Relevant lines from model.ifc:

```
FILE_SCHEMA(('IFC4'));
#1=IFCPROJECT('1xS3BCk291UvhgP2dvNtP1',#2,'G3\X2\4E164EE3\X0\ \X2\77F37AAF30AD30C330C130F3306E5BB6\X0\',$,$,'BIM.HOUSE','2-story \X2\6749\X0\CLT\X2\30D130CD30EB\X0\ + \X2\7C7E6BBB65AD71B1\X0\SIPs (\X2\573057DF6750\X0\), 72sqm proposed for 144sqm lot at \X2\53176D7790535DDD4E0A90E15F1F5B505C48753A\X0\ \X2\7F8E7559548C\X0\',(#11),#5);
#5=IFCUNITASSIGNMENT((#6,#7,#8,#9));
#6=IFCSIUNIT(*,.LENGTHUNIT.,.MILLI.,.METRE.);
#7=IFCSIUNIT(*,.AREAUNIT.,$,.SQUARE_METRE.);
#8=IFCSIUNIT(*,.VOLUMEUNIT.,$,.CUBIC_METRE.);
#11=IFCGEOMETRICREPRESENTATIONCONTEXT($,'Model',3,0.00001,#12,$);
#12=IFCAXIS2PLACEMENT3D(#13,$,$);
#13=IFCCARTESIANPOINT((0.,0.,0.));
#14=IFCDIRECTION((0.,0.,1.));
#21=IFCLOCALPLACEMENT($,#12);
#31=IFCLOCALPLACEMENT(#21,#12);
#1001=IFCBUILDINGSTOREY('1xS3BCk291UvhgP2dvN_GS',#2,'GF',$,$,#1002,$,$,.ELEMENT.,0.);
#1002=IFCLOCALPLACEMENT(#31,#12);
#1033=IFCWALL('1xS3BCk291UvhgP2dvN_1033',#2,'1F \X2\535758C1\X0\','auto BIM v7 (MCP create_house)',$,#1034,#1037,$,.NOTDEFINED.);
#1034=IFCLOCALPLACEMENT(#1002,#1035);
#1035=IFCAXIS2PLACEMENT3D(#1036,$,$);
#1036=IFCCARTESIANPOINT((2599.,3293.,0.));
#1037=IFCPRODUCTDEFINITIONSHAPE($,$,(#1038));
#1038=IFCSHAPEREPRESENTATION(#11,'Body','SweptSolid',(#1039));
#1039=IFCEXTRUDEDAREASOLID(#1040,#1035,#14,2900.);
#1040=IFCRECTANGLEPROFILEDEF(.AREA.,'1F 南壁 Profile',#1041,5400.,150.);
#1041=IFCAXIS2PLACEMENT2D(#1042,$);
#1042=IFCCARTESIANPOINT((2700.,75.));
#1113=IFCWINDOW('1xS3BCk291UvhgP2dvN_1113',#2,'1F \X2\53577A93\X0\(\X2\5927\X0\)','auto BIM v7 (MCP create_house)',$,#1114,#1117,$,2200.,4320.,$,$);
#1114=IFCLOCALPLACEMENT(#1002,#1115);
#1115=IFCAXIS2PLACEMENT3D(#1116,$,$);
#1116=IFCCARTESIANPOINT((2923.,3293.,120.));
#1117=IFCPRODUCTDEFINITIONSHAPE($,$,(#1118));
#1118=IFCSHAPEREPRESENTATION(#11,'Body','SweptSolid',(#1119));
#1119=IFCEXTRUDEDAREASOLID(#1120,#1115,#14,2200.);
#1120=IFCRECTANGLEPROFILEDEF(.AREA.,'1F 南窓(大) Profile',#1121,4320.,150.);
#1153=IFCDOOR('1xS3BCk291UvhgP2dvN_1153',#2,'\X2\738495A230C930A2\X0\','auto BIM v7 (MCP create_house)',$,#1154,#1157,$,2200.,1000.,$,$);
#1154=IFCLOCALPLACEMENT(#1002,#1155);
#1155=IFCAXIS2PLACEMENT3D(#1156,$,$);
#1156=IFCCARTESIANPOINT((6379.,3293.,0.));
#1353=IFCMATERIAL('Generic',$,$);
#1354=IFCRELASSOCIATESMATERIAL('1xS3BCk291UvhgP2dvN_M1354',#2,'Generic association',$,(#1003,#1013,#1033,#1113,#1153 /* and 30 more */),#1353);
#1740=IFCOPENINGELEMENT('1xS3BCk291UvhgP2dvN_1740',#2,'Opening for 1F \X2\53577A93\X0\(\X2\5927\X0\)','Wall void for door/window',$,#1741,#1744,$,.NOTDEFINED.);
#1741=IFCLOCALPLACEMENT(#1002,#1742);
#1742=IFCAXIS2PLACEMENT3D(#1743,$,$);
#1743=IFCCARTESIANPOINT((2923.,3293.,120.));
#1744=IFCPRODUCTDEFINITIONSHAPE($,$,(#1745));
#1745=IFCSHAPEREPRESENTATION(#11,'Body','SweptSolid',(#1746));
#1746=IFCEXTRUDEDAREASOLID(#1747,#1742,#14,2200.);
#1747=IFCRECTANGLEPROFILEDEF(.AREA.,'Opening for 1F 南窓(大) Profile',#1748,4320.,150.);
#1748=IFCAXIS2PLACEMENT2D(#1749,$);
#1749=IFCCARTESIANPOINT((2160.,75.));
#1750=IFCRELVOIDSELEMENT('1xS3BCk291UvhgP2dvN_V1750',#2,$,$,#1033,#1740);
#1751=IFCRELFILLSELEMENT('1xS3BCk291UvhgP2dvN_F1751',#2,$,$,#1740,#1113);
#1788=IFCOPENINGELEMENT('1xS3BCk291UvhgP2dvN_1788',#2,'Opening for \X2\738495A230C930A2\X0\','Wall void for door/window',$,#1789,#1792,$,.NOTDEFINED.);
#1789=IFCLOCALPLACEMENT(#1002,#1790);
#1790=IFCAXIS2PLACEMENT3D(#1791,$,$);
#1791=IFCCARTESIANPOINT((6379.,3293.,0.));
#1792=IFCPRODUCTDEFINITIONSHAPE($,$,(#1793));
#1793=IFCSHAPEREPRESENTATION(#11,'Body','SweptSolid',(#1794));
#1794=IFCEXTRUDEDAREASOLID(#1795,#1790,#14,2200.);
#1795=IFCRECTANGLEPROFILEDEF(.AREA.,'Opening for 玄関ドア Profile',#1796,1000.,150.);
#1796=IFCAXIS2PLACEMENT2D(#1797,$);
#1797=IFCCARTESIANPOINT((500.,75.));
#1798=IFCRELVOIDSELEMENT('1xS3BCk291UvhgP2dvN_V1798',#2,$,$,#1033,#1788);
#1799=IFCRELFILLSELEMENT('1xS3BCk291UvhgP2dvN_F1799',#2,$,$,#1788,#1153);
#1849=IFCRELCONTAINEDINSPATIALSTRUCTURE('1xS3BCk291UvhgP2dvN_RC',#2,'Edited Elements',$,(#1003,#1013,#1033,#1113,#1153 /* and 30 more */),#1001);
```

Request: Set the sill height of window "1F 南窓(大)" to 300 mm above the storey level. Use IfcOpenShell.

```python
import numpy as np
import ifcopenshell
import ifcopenshell.api.geometry
import ifcopenshell.geom
import ifcopenshell.util.element
import ifcopenshell.util.placement
import ifcopenshell.util.shape
import ifcopenshell.util.unit

model = ifcopenshell.open("model.ifc")
unit_scale = ifcopenshell.util.unit.calculate_unit_scale(model)

window = model.by_guid("1xS3BCk291UvhgP2dvN_1113")
opening = window.FillsVoids[0].RelatingOpeningElement
storey = ifcopenshell.util.element.get_container(window, ifc_class="IfcBuildingStorey")
level = ifcopenshell.util.placement.get_local_placement(storey.ObjectPlacement)[2, 3]

# The opening's origin need not be at the sill, so measure its lowest point.
shape = ifcopenshell.geom.create_shape(ifcopenshell.geom.settings(), opening)
bottom = ifcopenshell.util.shape.get_shape_bottom_elevation(shape, shape.geometry) / unit_scale
dz = level + 0.3 / unit_scale - bottom

shift = np.array([0.0, 0.0, dz])
# The window is not placed relative to its opening, so move both.
for product in (opening, window):
    matrix = ifcopenshell.util.placement.get_local_placement(product.ObjectPlacement)
    matrix[:3, 3] += shift
    ifcopenshell.api.geometry.edit_object_placement(model, product=product, matrix=matrix, is_si=False)

print(f"moved by {dz * unit_scale:+.3f} m")

model.write("model_v2.ifc")
```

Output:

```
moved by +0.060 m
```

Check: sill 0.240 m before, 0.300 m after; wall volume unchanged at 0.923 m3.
